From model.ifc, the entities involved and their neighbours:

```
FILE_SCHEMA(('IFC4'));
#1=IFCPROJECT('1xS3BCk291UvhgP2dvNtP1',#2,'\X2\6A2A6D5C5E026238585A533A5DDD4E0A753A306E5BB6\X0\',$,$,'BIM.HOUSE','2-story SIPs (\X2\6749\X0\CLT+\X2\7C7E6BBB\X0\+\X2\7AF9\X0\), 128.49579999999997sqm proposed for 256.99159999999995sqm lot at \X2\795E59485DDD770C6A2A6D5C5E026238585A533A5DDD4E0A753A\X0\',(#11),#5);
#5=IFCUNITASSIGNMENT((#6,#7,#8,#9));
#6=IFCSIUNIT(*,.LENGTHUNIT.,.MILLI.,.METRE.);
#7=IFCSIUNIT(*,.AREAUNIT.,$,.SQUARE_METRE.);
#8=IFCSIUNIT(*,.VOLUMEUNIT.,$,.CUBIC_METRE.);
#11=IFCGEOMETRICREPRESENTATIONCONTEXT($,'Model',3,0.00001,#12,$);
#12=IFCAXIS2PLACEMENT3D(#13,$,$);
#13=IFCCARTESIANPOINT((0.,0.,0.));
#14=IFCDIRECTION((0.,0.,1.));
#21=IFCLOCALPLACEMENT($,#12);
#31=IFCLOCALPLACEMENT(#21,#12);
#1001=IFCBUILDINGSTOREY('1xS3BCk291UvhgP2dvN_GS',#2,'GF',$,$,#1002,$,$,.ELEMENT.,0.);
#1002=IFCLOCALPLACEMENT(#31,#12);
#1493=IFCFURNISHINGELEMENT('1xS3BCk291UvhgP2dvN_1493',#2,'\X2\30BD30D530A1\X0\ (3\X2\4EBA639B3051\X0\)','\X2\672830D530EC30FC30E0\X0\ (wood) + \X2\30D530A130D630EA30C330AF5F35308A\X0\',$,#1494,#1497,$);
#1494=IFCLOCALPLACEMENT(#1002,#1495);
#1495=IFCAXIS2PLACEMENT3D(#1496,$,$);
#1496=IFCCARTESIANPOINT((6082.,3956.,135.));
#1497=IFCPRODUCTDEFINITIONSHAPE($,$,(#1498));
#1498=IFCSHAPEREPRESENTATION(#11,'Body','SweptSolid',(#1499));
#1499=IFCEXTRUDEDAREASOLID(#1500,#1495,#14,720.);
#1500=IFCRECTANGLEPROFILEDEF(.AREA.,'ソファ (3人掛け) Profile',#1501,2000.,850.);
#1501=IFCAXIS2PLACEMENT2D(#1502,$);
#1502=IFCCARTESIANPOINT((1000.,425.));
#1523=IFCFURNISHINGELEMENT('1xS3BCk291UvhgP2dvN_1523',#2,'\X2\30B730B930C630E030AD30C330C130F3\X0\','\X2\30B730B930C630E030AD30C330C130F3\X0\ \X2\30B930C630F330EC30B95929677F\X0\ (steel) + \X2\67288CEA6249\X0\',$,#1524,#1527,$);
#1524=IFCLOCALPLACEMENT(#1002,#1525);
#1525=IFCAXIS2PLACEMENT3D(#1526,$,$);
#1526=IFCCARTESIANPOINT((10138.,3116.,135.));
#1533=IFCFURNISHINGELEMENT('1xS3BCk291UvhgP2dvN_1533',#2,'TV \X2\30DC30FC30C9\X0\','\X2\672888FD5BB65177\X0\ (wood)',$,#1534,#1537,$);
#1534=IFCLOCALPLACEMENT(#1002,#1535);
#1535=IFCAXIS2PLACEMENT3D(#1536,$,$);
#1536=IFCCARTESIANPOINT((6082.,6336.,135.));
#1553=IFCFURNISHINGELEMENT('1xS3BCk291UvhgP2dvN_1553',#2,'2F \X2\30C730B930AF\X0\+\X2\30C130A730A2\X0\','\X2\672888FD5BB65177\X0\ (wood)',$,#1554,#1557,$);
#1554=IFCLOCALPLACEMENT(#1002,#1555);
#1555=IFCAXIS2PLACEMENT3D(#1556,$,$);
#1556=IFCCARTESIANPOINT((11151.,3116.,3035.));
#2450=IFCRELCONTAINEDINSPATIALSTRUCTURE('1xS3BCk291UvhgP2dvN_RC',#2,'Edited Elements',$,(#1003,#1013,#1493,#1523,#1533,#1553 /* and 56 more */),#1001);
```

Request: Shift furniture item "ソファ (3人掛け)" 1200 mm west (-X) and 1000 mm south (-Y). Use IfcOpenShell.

```python
import ifcopenshell
import ifcopenshell.api.geometry
import ifcopenshell.util.placement
import ifcopenshell.util.unit

model = ifcopenshell.open("model.ifc")
unit_scale = ifcopenshell.util.unit.calculate_unit_scale(model)

item = model.by_guid("1xS3BCk291UvhgP2dvN_1493")
matrix = ifcopenshell.util.placement.get_local_placement(item.ObjectPlacement)
matrix[0, 3] -= 1.2 / unit_scale
matrix[1, 3] -= 1 / unit_scale
ifcopenshell.api.geometry.edit_object_placement(model, product=item, matrix=matrix, is_si=False)

print(ifcopenshell.util.placement.get_local_placement(item.ObjectPlacement).round(3) + 0.0)

model.write("model-out.ifc")
```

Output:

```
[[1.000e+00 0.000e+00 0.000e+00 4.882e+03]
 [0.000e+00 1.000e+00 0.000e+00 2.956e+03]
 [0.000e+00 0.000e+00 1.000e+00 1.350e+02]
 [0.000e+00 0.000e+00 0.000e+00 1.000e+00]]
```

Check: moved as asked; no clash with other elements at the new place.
